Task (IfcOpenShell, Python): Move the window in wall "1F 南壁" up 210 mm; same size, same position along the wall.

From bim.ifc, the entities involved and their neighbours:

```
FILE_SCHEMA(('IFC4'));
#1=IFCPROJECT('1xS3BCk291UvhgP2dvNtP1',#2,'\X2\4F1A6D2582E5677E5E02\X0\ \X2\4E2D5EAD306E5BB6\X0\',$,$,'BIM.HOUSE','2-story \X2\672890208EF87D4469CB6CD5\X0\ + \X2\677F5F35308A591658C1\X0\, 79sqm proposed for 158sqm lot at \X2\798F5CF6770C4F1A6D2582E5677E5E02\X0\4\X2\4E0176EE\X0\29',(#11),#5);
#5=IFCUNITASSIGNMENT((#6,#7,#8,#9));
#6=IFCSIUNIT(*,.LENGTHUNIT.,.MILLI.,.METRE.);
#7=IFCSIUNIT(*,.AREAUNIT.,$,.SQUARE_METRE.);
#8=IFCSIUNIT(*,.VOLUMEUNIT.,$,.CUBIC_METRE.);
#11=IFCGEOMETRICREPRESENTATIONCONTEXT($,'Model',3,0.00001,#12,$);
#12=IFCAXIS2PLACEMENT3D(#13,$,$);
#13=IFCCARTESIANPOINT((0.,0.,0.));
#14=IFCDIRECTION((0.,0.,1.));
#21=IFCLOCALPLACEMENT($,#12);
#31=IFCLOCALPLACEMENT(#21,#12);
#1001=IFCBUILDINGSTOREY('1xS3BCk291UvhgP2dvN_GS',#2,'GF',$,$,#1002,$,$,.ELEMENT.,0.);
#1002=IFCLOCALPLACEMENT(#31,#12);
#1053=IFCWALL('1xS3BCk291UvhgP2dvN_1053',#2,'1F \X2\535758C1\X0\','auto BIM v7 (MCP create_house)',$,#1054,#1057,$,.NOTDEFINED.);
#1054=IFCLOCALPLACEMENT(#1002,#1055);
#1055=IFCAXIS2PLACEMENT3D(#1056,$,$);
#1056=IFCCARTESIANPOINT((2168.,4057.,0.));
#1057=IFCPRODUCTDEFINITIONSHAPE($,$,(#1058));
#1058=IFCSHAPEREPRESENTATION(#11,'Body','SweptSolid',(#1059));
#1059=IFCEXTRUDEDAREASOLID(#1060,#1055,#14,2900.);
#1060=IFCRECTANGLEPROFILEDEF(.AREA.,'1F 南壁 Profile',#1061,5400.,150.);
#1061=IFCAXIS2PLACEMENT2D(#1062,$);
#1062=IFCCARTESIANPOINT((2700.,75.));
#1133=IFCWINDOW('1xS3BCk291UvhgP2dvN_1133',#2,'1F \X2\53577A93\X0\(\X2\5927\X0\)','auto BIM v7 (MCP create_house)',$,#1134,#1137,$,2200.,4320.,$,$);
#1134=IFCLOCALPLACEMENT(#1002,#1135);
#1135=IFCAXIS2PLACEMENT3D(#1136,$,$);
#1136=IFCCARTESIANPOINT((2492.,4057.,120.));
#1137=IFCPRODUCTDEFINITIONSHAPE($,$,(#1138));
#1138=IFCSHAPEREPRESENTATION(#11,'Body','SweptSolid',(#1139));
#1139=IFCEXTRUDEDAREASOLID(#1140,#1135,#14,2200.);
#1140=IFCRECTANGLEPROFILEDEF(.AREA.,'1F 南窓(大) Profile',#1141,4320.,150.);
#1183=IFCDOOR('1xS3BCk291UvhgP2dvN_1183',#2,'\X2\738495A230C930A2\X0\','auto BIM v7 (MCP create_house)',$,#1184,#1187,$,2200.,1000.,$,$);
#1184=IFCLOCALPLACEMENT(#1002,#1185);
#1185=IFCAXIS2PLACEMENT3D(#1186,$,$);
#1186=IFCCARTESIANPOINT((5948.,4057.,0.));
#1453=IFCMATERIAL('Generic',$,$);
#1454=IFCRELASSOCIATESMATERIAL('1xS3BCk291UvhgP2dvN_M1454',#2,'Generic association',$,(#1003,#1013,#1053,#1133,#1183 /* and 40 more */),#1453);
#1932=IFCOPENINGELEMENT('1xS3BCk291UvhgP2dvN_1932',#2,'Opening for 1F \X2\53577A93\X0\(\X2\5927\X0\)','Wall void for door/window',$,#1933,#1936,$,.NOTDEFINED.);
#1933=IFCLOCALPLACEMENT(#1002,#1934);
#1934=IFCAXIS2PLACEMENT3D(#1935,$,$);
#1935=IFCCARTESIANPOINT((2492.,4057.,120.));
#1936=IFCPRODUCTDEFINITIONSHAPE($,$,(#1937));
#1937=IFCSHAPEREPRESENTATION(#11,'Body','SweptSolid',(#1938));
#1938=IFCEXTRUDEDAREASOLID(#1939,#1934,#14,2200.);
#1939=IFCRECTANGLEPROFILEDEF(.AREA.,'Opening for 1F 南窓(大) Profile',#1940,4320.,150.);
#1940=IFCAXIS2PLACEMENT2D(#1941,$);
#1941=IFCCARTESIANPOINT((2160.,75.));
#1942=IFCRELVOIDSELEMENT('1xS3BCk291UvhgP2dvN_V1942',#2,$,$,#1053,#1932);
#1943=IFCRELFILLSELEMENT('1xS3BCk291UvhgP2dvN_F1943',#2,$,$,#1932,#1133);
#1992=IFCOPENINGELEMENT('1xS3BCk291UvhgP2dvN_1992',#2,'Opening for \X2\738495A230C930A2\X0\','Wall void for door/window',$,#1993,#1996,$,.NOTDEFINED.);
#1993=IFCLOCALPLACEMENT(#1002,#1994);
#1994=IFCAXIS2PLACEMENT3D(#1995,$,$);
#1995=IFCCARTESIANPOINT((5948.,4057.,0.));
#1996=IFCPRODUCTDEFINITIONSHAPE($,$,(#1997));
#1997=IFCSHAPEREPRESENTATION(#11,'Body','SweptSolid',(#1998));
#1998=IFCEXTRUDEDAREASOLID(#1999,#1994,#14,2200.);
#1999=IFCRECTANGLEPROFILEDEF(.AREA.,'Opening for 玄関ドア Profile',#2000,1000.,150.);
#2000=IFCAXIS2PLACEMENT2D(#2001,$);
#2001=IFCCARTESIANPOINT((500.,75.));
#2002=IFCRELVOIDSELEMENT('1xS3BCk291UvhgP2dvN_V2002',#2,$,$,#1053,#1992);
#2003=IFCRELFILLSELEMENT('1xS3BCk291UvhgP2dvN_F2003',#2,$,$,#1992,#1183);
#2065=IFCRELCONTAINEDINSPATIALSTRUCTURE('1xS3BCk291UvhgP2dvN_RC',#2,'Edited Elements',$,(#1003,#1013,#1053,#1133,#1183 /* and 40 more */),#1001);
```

```python
import numpy as np
import ifcopenshell
import ifcopenshell.api.geometry
import ifcopenshell.util.placement
import ifcopenshell.util.unit

model = ifcopenshell.open("bim.ifc")
unit_scale = ifcopenshell.util.unit.calculate_unit_scale(model)

window = model.by_guid("1xS3BCk291UvhgP2dvN_1133")
opening = window.FillsVoids[0].RelatingOpeningElement
dz = 210.0

shift = np.array([0.0, 0.0, dz])
# The window is not placed relative to its opening, so move both.
for product in (opening, window):
    matrix = ifcopenshell.util.placement.get_local_placement(product.ObjectPlacement)
    matrix[:3, 3] += shift
    ifcopenshell.api.geometry.edit_object_placement(model, product=product, matrix=matrix, is_si=False)

print(f"moved by {dz * unit_scale:+.3f} m")

model.write("bim_rev.ifc")
```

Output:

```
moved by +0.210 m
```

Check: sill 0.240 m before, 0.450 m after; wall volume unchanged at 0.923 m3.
